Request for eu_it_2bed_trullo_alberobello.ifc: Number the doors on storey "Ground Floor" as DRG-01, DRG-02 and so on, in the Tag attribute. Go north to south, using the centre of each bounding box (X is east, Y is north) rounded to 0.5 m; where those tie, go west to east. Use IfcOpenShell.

First a look at what the model holds.

```python
import ifcopenshell
import ifcopenshell.util.element
import ifcopenshell.util.placement

model = ifcopenshell.open("eu_it_2bed_trullo_alberobello.ifc")
print(model.schema)
storey = next(s for s in model.by_type("IfcBuildingStorey") if s.Name == "Ground Floor")
doors = [e for e in ifcopenshell.util.element.get_decomposition(storey) if e.is_a("IfcDoor")]
for e in sorted(doors, key=lambda e: e.id()):
    origin = ifcopenshell.util.placement.get_local_placement(e.ObjectPlacement)[:3, 3]
    print(e.id(), e.Tag, e.Name, origin.round(2) + 0.0, sep=" | ")
```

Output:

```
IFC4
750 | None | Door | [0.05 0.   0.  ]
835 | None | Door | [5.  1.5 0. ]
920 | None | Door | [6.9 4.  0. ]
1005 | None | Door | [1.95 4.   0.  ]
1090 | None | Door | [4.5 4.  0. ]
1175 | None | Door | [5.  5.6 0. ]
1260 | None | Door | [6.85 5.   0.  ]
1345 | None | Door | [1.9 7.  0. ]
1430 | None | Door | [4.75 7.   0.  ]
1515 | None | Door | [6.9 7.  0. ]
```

```python
import ifcopenshell
import ifcopenshell.geom
import ifcopenshell.util.element
import ifcopenshell.util.shape

model = ifcopenshell.open("eu_it_2bed_trullo_alberobello.ifc")
settings = ifcopenshell.geom.settings()
settings.set("use-world-coords", True)


def centre(element):
    shape = ifcopenshell.geom.create_shape(settings, element)
    return ifcopenshell.util.shape.get_bbox_centroid(shape.geometry)


storey = next(s for s in model.by_type("IfcBuildingStorey") if s.Name == "Ground Floor")
doors = [e for e in ifcopenshell.util.element.get_decomposition(storey) if e.is_a("IfcDoor")]

# Insertion points can sit at a corner or the storey origin, so sort by the geometry (in metres).
centres = {e: centre(e) for e in doors}
doors.sort(key=lambda e: (-round(centres[e][1] / 0.5), centres[e][0]))

for i, e in enumerate(doors, start=1):
    number = f"DRG-{i:02d}"
    e.Tag = number
    print(e.id(), number)

model.write("eu_it_2bed_trullo_alberobello_updated.ifc")
```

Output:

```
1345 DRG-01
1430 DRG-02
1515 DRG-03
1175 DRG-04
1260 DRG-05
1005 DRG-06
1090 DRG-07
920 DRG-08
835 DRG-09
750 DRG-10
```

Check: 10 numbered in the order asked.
